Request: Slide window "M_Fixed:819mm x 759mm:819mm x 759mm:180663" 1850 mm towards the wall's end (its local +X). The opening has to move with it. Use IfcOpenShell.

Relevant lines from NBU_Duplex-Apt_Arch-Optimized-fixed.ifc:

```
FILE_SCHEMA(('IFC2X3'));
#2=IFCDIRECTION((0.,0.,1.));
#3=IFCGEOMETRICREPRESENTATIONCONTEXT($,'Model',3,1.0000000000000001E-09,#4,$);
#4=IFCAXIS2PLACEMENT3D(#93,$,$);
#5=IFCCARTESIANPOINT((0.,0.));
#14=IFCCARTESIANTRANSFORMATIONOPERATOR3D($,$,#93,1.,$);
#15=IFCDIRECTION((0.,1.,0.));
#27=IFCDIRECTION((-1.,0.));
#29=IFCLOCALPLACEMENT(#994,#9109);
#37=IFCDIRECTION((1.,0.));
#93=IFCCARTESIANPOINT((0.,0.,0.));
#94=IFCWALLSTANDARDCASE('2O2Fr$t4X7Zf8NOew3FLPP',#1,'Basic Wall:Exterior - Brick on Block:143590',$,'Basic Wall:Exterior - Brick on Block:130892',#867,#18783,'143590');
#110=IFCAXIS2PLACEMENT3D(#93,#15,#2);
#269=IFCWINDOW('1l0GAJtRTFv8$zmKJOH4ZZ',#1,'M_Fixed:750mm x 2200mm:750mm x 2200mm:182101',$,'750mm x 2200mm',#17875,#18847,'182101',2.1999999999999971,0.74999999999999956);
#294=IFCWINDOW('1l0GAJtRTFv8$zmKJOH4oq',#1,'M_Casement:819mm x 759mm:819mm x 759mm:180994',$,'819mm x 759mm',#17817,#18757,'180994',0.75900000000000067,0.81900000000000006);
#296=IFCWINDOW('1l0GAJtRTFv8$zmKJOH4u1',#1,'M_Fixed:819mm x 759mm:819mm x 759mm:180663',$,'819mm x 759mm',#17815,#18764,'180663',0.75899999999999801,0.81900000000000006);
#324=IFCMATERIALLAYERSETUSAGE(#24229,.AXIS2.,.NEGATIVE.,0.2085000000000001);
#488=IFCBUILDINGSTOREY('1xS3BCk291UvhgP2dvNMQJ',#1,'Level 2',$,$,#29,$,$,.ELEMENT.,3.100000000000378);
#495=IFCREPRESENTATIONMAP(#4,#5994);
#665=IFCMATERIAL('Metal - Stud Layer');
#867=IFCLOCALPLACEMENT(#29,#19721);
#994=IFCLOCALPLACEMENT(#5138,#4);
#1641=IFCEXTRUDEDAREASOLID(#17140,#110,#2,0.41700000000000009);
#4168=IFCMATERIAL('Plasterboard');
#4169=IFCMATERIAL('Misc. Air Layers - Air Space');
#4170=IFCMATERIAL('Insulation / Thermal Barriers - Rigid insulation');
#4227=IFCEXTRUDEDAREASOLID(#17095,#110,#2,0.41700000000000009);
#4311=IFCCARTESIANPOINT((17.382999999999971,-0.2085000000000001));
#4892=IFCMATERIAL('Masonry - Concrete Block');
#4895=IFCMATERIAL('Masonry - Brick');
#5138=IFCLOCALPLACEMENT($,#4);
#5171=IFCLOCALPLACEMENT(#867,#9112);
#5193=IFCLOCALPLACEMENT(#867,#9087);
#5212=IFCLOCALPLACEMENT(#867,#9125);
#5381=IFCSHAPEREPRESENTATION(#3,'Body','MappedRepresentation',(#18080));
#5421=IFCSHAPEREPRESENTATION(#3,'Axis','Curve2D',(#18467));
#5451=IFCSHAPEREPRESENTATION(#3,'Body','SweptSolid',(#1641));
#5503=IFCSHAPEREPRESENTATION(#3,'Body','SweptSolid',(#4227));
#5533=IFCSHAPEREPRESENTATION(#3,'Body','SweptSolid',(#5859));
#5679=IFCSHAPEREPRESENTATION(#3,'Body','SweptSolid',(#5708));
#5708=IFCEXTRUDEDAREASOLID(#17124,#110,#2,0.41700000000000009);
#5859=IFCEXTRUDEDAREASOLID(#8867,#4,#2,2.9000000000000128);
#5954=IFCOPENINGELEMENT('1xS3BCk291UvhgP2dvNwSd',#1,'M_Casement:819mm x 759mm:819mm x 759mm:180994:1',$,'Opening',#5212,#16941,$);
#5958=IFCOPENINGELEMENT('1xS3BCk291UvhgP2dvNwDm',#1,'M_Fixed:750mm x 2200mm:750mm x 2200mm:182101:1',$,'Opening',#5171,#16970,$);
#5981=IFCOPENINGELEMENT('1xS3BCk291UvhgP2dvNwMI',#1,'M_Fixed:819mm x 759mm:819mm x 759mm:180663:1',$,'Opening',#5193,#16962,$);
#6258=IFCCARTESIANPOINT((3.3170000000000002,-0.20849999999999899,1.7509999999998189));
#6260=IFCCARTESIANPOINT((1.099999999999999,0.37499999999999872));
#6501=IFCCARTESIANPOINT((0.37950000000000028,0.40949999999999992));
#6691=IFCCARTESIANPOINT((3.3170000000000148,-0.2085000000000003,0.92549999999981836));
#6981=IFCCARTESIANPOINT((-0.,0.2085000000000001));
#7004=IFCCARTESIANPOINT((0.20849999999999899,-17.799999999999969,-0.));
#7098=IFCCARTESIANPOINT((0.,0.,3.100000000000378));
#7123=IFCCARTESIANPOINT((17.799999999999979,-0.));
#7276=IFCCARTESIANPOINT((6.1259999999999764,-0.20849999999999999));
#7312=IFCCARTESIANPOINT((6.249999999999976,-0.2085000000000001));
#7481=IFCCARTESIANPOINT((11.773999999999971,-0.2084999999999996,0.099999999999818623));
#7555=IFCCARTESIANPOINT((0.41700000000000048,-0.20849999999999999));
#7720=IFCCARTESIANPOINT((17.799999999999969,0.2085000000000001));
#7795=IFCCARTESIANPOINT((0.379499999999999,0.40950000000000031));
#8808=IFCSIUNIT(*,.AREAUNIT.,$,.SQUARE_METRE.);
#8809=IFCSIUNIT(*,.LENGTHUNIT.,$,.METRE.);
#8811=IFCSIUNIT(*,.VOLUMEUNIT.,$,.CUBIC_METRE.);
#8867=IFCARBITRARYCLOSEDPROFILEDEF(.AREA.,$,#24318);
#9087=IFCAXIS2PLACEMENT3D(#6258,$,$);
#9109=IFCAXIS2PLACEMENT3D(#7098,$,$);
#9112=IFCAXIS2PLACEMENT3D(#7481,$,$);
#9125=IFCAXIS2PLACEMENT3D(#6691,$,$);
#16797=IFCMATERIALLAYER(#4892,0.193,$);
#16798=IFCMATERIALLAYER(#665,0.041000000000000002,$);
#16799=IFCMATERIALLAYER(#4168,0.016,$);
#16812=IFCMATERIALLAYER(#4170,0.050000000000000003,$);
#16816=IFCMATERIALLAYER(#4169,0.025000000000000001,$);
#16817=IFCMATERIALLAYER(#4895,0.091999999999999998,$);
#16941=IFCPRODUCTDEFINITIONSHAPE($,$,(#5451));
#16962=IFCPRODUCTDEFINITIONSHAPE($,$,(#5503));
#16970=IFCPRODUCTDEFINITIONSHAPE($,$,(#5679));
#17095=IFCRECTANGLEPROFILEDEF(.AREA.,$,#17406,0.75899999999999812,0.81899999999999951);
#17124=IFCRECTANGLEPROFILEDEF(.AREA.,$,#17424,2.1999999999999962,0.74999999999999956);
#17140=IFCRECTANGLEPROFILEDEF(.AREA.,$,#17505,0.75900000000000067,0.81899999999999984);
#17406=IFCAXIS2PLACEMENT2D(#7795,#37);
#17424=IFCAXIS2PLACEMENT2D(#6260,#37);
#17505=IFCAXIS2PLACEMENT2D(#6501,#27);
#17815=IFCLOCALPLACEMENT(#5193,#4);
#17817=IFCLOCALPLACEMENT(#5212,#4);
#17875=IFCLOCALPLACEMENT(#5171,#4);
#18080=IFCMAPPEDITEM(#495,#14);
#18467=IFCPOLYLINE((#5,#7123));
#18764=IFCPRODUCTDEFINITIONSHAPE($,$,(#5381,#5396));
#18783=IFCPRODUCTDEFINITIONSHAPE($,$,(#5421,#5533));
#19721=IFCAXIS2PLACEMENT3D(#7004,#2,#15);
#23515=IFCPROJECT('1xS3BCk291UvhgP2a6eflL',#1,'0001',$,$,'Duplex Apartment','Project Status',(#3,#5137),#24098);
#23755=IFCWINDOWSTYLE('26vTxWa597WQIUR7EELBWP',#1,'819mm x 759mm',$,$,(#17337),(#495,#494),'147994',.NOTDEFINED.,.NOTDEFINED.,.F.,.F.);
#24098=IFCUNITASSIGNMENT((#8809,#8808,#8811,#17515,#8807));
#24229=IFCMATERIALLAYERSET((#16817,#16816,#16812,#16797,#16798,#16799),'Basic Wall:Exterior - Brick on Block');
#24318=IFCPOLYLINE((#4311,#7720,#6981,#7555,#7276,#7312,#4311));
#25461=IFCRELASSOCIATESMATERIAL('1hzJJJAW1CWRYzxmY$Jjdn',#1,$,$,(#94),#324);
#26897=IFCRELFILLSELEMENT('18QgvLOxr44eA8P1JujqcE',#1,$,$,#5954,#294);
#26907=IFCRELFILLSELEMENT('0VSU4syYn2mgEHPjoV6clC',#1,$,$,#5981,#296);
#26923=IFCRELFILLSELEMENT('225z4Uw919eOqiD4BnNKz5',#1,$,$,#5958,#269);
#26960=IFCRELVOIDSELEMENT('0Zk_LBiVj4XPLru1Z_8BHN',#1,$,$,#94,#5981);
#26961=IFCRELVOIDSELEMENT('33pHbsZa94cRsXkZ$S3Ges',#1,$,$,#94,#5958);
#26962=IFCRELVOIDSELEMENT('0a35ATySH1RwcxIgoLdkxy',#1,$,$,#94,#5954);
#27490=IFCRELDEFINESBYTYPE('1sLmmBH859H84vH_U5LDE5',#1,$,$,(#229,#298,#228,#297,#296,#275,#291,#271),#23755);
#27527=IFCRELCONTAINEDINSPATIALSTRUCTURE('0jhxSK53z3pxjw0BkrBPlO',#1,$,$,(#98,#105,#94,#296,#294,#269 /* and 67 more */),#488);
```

```python
import ifcopenshell
import ifcopenshell.api.geometry
import ifcopenshell.util.placement

model = ifcopenshell.open("NBU_Duplex-Apt_Arch-Optimized-fixed.ifc")

window = model.by_guid("1l0GAJtRTFv8$zmKJOH4u1")
opening = window.FillsVoids[0].RelatingOpeningElement
wall = opening.VoidsElements[0].RelatingBuildingElement

wall_matrix = ifcopenshell.util.placement.get_local_placement(wall.ObjectPlacement)
shift = wall_matrix[:3, 0] * 1.85
before = ifcopenshell.util.placement.get_local_placement(window.ObjectPlacement)[:3, 3].copy()

# The window is placed relative to its opening, so it follows when the opening moves.
matrix = ifcopenshell.util.placement.get_local_placement(opening.ObjectPlacement)
matrix[:3, 3] += shift
ifcopenshell.api.geometry.edit_object_placement(
    model, product=opening, matrix=matrix, is_si=False, should_transform_children=True
)

after = ifcopenshell.util.placement.get_local_placement(window.ObjectPlacement)[:3, 3]
print("window moved by", (after - before).round(3) + 0.0)

model.write("NBU_Duplex-Apt_Arch-Optimized-fixed_rev.ifc")
```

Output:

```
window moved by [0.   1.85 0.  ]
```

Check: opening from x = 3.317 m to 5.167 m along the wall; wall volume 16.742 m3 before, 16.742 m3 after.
